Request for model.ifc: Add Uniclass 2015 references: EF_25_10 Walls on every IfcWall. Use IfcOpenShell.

First a look at what the model holds.

```python
import ifcopenshell

model = ifcopenshell.open("model.ifc")
print(model.schema)
print("classifications:", [c.Name for c in model.by_type("IfcClassification")])
for ifc_class in ("IfcDoor", "IfcRoof", "IfcStair", "IfcWall", "IfcWindow"):
    print(ifc_class, len(model.by_type(ifc_class)))
```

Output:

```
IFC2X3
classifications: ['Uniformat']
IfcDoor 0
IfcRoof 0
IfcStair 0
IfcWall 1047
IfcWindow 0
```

```python
import ifcopenshell
import ifcopenshell.api.classification

model = ifcopenshell.open("model.ifc")

# IFC2X3 requires Source and Edition and has no link from the project to the system.
system = model.create_entity("IfcClassification", Source="NBS", Edition="2015", Name="Uniclass 2015")

codes = {
    "IfcWall": ("EF_25_10", "Walls"),
}
for ifc_class, (code, name) in codes.items():
    products = model.by_type(ifc_class)
    ifcopenshell.api.classification.add_reference(
        model, products=products, classification=system, identification=code, name=name
    )
    print(code, len(products))

model.write("model-out.ifc")
```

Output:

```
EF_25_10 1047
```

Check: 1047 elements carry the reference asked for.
